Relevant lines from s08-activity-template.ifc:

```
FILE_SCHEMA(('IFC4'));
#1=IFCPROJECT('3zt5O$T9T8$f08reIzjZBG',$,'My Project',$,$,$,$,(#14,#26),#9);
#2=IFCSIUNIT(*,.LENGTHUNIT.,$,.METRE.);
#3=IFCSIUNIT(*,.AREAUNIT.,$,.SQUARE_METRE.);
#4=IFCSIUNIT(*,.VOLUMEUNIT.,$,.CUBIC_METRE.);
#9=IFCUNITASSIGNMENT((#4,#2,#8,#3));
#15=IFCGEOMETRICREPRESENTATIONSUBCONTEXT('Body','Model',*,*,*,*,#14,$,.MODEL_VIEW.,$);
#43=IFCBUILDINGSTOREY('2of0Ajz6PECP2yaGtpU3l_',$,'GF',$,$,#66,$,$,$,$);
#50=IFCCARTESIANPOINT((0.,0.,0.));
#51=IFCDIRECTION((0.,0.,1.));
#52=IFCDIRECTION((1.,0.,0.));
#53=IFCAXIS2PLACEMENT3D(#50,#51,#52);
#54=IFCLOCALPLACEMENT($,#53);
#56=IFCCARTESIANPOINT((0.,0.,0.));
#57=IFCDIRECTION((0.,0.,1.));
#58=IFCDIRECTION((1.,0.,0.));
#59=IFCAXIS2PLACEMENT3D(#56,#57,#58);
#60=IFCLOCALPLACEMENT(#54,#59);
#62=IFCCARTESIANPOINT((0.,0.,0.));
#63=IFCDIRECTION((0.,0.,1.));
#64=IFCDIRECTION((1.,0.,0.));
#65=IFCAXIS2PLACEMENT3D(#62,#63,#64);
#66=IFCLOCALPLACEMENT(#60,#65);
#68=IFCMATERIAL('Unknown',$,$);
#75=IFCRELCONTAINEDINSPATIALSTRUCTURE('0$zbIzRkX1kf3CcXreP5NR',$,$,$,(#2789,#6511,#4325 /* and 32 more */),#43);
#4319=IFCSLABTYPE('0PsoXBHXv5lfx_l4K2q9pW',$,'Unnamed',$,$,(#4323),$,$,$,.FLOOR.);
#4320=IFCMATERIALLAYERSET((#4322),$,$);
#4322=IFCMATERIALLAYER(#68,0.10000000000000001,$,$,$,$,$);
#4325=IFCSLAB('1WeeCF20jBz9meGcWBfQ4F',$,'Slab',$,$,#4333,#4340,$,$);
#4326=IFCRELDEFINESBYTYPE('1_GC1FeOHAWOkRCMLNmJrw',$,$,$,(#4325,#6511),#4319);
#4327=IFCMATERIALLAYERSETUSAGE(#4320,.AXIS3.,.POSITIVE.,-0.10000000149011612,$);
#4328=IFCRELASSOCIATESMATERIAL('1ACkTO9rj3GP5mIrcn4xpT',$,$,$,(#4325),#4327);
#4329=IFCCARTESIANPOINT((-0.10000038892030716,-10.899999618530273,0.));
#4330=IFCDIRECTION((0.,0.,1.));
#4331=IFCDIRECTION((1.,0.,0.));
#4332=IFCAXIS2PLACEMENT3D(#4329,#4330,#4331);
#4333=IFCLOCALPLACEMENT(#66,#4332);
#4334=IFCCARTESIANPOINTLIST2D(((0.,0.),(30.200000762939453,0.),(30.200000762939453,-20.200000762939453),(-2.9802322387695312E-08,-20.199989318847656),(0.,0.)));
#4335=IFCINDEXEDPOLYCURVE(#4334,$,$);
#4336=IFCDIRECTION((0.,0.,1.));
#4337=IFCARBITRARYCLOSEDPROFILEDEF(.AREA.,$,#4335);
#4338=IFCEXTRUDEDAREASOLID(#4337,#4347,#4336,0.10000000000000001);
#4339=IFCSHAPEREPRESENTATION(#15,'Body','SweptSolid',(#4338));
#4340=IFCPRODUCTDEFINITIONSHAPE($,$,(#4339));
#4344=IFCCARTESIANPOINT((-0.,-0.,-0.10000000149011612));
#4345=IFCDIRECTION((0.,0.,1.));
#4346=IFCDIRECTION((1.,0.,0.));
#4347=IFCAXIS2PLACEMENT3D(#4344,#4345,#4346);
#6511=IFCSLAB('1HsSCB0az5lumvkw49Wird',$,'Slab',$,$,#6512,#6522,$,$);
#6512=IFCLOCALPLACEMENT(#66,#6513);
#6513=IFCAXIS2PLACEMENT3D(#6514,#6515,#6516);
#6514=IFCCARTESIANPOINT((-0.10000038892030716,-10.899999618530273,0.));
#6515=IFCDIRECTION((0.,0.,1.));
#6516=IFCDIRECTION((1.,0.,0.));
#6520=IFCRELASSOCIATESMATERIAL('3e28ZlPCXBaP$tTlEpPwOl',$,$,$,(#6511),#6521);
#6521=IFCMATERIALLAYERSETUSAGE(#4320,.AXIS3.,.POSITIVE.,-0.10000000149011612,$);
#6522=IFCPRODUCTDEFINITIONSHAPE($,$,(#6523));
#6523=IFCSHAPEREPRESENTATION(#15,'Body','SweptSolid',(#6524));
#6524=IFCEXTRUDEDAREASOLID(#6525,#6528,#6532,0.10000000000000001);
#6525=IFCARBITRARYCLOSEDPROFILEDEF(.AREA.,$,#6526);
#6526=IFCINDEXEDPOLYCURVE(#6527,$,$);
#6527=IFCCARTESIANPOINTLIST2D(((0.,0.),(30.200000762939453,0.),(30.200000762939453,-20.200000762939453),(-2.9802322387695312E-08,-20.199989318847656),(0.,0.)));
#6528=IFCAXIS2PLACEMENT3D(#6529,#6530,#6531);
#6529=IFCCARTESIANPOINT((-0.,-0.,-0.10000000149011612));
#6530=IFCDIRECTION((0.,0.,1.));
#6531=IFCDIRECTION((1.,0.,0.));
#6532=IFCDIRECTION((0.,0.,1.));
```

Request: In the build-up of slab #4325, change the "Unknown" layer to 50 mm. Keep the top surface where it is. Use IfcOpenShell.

```python
import ifcopenshell
import ifcopenshell.util.element
import ifcopenshell.util.representation

model = ifcopenshell.open("s08-activity-template.ifc")

layer_set = model.by_id(4320)
layer = next(l for l in layer_set.MaterialLayers if l.Material and l.Material.Name == "Unknown")
change = 0.05 - layer.LayerThickness
layer.LayerThickness += change

# The layer set is shared, so every slab that uses it gets the new thickness.
slabs = [e for e in ifcopenshell.util.element.get_elements_by_material(model, layer_set) if e.is_a("IfcSlab")]
for slab in sorted(slabs, key=lambda e: e.id()):
    body = ifcopenshell.util.representation.get_representation(slab, "Model", "Body")
    solid = body.Items[0]
    old_depth = solid.Depth
    solid.Depth += change
    # Extruded upwards: lower the start of the extrusion so the top stays.
    x, y, z = solid.Position.Location.Coordinates
    solid.Position.Location = model.createIfcCartesianPoint((x, y, z - change))
    print(slab.id(), f"{old_depth:g} -> {solid.Depth:g}")

# The layers are counted up from the underside, which has moved.
for usage in {ifcopenshell.util.element.get_material(slab) for slab in slabs}:
    usage.OffsetFromReferenceLine -= change

model.write("s08-activity-template_edited.ifc")
```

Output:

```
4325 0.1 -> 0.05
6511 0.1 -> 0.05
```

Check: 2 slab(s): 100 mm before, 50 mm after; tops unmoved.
